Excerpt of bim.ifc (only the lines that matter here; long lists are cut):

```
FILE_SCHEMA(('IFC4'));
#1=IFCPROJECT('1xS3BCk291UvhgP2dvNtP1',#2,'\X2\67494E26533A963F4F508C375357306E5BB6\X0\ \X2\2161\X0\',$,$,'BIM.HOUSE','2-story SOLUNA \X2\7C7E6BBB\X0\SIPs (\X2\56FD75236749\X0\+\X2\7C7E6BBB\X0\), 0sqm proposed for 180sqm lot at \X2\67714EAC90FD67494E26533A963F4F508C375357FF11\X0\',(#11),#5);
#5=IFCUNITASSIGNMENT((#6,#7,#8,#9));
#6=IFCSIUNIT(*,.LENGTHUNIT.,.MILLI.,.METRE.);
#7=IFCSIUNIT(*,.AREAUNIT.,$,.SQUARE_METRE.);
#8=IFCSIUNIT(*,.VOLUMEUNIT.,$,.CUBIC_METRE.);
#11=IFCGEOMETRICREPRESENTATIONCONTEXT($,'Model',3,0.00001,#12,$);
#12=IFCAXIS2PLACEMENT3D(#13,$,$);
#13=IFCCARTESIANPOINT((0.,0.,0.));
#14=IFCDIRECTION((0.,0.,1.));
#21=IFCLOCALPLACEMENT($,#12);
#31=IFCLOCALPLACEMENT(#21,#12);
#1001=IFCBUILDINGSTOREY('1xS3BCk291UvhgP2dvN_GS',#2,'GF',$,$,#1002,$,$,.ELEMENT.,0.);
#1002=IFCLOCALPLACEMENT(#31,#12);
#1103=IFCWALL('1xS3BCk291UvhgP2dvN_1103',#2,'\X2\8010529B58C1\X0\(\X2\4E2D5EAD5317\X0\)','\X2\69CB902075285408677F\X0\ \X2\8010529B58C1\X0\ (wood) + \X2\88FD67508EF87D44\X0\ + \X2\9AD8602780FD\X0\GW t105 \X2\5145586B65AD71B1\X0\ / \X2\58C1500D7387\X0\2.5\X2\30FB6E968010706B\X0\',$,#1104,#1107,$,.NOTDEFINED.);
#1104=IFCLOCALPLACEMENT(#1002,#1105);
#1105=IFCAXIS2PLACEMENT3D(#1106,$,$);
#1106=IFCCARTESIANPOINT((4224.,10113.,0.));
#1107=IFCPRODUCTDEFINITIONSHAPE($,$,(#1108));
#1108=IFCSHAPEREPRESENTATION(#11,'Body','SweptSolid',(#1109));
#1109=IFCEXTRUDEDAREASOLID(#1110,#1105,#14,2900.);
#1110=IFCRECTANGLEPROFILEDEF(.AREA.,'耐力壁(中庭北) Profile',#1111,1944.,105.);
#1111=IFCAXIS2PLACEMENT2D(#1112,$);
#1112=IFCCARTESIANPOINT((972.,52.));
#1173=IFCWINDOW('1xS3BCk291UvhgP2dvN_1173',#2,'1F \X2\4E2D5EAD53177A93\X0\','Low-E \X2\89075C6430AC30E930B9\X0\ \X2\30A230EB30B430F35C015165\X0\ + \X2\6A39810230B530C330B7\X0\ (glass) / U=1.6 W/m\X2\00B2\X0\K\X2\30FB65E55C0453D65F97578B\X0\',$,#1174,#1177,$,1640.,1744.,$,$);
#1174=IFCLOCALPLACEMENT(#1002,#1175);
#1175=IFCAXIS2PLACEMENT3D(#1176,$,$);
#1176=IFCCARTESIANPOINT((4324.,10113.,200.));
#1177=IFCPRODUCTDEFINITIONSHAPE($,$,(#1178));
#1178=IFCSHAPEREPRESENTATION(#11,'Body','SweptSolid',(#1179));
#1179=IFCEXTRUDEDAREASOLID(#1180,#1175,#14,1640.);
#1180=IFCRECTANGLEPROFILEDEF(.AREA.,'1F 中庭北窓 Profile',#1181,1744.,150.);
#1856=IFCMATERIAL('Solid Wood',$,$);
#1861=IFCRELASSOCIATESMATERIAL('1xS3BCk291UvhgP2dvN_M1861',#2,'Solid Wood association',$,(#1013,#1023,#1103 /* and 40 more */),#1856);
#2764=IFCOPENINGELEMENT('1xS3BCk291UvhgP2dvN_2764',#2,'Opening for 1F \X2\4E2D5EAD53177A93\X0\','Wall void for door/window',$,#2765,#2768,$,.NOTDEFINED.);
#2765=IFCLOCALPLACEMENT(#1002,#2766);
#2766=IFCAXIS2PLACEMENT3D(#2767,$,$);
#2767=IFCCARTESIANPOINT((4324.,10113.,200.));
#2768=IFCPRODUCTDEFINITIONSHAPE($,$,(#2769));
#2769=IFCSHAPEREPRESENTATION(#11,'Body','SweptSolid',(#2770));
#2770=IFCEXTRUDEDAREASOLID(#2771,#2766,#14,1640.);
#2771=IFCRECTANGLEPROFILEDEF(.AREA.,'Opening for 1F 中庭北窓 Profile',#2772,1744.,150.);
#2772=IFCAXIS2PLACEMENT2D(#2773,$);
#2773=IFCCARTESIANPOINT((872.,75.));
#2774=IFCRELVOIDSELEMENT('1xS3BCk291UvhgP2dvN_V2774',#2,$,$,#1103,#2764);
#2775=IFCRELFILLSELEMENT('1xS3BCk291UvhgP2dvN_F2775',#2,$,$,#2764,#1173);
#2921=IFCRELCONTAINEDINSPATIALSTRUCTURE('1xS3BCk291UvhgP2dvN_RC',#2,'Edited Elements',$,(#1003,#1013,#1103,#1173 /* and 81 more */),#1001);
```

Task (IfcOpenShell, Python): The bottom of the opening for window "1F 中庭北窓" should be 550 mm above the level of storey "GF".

```python
import numpy as np
import ifcopenshell
import ifcopenshell.api.geometry
import ifcopenshell.geom
import ifcopenshell.util.element
import ifcopenshell.util.placement
import ifcopenshell.util.shape
import ifcopenshell.util.unit

model = ifcopenshell.open("bim.ifc")
unit_scale = ifcopenshell.util.unit.calculate_unit_scale(model)

window = model.by_id(1173)
opening = window.FillsVoids[0].RelatingOpeningElement
storey = ifcopenshell.util.element.get_container(window, ifc_class="IfcBuildingStorey")
level = ifcopenshell.util.placement.get_local_placement(storey.ObjectPlacement)[2, 3]

# The opening's origin need not be at the sill, so measure its lowest point.
shape = ifcopenshell.geom.create_shape(ifcopenshell.geom.settings(), opening)
bottom = ifcopenshell.util.shape.get_shape_bottom_elevation(shape, shape.geometry) / unit_scale
dz = level + 550.0 - bottom

shift = np.array([0.0, 0.0, dz])
# The window is not placed relative to its opening, so move both.
for product in (opening, window):
    matrix = ifcopenshell.util.placement.get_local_placement(product.ObjectPlacement)
    matrix[:3, 3] += shift
    ifcopenshell.api.geometry.edit_object_placement(model, product=product, matrix=matrix, is_si=False)

print(f"moved by {dz * unit_scale:+.3f} m")

model.write("bim_v2.ifc")
```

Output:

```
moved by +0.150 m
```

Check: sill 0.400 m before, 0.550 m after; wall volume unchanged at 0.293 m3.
